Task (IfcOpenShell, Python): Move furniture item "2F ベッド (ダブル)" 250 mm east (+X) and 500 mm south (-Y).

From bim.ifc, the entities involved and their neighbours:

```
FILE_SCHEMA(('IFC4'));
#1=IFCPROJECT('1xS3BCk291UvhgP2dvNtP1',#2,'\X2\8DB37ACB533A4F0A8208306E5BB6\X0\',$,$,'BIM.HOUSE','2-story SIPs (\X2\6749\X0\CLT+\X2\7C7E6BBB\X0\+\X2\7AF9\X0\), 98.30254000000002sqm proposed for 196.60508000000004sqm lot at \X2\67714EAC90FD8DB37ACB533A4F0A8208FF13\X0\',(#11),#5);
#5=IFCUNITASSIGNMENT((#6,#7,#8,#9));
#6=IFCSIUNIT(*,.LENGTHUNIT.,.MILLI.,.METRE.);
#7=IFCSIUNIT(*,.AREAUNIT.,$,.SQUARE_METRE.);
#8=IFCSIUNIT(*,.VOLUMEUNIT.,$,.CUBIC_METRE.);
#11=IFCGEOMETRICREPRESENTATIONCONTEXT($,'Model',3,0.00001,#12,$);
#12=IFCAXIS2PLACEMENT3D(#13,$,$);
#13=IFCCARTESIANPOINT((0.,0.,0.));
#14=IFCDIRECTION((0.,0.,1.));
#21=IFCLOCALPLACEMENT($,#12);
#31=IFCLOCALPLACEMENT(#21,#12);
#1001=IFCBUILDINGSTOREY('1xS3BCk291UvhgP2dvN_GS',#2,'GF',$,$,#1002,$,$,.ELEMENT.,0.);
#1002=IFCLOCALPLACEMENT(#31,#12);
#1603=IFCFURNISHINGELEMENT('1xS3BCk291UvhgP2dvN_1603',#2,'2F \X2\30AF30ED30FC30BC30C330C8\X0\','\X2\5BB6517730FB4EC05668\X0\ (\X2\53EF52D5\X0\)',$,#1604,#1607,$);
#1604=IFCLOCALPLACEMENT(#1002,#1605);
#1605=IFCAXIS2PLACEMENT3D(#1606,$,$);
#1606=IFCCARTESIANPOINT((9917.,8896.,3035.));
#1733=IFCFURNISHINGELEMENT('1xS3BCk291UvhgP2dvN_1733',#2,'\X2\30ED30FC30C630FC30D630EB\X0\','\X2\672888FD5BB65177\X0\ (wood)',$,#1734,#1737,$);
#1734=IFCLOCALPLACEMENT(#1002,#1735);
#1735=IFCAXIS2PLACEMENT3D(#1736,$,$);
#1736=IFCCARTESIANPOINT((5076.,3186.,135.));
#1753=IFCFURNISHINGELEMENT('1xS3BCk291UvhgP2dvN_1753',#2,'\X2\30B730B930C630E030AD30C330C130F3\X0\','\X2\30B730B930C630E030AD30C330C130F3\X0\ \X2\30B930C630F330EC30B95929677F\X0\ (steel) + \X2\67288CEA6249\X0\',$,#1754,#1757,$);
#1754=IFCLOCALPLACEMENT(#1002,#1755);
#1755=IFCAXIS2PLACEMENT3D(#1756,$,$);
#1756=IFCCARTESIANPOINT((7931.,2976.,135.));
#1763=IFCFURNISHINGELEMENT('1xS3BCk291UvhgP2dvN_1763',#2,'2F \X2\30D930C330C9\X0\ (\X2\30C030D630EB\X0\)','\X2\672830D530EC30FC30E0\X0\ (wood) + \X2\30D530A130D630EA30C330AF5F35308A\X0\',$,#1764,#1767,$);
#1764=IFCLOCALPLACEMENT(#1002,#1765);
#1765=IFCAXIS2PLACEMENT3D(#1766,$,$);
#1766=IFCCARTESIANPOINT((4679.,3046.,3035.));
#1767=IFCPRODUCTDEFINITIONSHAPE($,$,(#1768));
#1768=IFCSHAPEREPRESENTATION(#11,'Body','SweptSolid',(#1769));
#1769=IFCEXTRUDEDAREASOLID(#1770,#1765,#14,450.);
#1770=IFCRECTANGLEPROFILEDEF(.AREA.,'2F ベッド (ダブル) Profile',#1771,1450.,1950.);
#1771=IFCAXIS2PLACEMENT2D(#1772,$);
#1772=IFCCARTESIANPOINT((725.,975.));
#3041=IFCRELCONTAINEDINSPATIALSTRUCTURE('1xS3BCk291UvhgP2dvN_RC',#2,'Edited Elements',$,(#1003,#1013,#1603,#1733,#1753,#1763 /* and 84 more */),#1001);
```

```python
import ifcopenshell
import ifcopenshell.api.geometry
import ifcopenshell.util.placement

model = ifcopenshell.open("bim.ifc")

item = model.by_guid("1xS3BCk291UvhgP2dvN_1763")
matrix = ifcopenshell.util.placement.get_local_placement(item.ObjectPlacement)
matrix[0, 3] += 250.0
matrix[1, 3] -= 500.0
ifcopenshell.api.geometry.edit_object_placement(model, product=item, matrix=matrix, is_si=False)

print(ifcopenshell.util.placement.get_local_placement(item.ObjectPlacement).round(3) + 0.0)

model.write("bim_updated.ifc")
```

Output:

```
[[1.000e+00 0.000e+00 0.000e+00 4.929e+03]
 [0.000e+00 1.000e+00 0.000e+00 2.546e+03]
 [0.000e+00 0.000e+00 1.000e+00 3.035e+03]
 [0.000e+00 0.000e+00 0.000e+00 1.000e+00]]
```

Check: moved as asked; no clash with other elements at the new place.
